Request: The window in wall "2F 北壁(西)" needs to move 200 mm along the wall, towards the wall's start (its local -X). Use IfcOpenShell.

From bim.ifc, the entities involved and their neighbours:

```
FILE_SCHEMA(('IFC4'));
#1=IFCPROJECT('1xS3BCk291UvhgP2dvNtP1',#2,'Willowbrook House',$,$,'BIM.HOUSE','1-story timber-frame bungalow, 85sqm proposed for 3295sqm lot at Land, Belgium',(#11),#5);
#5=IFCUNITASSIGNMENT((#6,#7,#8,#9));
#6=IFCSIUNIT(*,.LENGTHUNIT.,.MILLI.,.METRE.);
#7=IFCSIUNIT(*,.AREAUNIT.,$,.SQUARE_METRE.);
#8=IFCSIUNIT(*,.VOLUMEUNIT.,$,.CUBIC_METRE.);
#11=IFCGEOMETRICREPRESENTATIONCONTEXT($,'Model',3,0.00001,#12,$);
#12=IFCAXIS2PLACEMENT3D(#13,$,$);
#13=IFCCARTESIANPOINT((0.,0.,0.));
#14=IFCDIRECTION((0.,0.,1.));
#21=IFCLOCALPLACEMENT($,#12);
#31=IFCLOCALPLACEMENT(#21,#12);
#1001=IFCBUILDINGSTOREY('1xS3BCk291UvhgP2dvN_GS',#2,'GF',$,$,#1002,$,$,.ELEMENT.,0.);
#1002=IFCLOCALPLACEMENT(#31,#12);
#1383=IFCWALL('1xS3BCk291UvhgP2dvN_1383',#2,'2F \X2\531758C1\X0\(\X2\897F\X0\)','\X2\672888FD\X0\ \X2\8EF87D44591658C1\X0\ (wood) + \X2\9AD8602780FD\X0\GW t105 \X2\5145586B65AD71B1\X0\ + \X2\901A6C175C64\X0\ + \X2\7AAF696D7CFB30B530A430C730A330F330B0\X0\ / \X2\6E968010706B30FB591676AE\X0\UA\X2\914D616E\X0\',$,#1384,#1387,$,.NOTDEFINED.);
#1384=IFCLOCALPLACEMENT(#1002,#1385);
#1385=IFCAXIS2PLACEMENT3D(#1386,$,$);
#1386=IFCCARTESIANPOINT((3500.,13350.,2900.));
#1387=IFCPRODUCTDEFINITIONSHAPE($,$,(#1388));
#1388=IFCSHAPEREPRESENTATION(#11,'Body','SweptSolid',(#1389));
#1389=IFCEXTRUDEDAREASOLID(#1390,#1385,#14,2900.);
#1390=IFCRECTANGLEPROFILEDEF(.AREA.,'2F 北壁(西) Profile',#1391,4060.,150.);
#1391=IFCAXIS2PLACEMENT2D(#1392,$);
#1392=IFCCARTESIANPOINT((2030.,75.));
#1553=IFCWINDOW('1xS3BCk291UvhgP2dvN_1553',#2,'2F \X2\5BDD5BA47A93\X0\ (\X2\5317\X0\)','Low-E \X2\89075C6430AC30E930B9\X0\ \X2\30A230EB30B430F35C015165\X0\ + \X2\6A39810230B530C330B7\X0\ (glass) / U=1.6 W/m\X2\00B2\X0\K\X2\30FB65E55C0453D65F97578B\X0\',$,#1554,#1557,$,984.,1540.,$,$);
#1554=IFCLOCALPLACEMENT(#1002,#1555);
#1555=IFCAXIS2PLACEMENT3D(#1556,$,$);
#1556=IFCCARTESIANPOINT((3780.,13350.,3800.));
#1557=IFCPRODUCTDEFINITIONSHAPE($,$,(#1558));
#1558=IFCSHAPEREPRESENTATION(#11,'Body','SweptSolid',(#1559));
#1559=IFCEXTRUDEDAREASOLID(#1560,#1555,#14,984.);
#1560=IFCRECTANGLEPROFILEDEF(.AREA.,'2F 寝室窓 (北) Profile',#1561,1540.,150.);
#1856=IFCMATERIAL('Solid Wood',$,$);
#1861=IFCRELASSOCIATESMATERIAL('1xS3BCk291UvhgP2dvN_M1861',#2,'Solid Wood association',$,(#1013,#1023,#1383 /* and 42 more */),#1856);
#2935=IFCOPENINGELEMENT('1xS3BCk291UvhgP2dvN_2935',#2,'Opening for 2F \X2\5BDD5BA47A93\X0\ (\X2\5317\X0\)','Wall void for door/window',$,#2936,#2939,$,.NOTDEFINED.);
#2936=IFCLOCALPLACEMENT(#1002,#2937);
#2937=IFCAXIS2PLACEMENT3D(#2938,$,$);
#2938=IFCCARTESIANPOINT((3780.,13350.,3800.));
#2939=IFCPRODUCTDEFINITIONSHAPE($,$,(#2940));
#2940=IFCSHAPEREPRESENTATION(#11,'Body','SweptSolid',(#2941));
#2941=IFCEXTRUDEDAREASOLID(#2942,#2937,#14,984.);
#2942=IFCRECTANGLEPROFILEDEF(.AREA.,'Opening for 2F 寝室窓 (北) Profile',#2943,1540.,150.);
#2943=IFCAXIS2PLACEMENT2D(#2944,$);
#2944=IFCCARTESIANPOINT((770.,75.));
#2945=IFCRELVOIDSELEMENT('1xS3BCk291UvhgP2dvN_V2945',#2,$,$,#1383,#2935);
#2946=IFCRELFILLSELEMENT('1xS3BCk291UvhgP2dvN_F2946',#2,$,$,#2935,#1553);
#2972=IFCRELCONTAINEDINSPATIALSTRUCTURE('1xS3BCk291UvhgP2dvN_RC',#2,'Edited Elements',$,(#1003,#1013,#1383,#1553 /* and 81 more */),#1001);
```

```python
import ifcopenshell
import ifcopenshell.api.geometry
import ifcopenshell.util.placement

model = ifcopenshell.open("bim.ifc")

window = model.by_guid("1xS3BCk291UvhgP2dvN_1553")
opening = window.FillsVoids[0].RelatingOpeningElement
wall = opening.VoidsElements[0].RelatingBuildingElement

wall_matrix = ifcopenshell.util.placement.get_local_placement(wall.ObjectPlacement)
shift = wall_matrix[:3, 0] * -200.0
before = ifcopenshell.util.placement.get_local_placement(window.ObjectPlacement)[:3, 3].copy()

# The window is not placed relative to its opening, so move both.
for product in (opening, window):
    matrix = ifcopenshell.util.placement.get_local_placement(product.ObjectPlacement)
    matrix[:3, 3] += shift
    ifcopenshell.api.geometry.edit_object_placement(model, product=product, matrix=matrix, is_si=False)

after = ifcopenshell.util.placement.get_local_placement(window.ObjectPlacement)[:3, 3]
print("window moved by", (after - before).round(3) + 0.0)

model.write("bim_v2.ifc")
```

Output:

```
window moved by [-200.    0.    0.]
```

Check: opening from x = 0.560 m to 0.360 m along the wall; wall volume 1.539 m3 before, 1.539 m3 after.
